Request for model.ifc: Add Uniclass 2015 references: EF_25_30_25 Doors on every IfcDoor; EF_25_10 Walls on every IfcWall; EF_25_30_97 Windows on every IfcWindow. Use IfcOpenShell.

First a look at what the model holds.

```python
import ifcopenshell

model = ifcopenshell.open("model.ifc")
print(model.schema)
print("classifications:", [c.Name for c in model.by_type("IfcClassification")])
for ifc_class in ("IfcDoor", "IfcRoof", "IfcStair", "IfcWall", "IfcWindow"):
    print(ifc_class, len(model.by_type(ifc_class)))
```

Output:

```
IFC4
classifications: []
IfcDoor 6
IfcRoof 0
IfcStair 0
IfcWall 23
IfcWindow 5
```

```python
import ifcopenshell
import ifcopenshell.api.classification

model = ifcopenshell.open("model.ifc")

system = ifcopenshell.api.classification.add_classification(model, classification="Uniclass 2015")

codes = {
    "IfcDoor": ("EF_25_30_25", "Doors"),
    "IfcWall": ("EF_25_10", "Walls"),
    "IfcWindow": ("EF_25_30_97", "Windows"),
}
for ifc_class, (code, name) in codes.items():
    products = model.by_type(ifc_class)
    ifcopenshell.api.classification.add_reference(
        model, products=products, classification=system, identification=code, name=name
    )
    print(code, len(products))

model.write("model_updated.ifc")
```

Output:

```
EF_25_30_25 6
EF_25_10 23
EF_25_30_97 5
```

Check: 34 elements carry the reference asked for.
